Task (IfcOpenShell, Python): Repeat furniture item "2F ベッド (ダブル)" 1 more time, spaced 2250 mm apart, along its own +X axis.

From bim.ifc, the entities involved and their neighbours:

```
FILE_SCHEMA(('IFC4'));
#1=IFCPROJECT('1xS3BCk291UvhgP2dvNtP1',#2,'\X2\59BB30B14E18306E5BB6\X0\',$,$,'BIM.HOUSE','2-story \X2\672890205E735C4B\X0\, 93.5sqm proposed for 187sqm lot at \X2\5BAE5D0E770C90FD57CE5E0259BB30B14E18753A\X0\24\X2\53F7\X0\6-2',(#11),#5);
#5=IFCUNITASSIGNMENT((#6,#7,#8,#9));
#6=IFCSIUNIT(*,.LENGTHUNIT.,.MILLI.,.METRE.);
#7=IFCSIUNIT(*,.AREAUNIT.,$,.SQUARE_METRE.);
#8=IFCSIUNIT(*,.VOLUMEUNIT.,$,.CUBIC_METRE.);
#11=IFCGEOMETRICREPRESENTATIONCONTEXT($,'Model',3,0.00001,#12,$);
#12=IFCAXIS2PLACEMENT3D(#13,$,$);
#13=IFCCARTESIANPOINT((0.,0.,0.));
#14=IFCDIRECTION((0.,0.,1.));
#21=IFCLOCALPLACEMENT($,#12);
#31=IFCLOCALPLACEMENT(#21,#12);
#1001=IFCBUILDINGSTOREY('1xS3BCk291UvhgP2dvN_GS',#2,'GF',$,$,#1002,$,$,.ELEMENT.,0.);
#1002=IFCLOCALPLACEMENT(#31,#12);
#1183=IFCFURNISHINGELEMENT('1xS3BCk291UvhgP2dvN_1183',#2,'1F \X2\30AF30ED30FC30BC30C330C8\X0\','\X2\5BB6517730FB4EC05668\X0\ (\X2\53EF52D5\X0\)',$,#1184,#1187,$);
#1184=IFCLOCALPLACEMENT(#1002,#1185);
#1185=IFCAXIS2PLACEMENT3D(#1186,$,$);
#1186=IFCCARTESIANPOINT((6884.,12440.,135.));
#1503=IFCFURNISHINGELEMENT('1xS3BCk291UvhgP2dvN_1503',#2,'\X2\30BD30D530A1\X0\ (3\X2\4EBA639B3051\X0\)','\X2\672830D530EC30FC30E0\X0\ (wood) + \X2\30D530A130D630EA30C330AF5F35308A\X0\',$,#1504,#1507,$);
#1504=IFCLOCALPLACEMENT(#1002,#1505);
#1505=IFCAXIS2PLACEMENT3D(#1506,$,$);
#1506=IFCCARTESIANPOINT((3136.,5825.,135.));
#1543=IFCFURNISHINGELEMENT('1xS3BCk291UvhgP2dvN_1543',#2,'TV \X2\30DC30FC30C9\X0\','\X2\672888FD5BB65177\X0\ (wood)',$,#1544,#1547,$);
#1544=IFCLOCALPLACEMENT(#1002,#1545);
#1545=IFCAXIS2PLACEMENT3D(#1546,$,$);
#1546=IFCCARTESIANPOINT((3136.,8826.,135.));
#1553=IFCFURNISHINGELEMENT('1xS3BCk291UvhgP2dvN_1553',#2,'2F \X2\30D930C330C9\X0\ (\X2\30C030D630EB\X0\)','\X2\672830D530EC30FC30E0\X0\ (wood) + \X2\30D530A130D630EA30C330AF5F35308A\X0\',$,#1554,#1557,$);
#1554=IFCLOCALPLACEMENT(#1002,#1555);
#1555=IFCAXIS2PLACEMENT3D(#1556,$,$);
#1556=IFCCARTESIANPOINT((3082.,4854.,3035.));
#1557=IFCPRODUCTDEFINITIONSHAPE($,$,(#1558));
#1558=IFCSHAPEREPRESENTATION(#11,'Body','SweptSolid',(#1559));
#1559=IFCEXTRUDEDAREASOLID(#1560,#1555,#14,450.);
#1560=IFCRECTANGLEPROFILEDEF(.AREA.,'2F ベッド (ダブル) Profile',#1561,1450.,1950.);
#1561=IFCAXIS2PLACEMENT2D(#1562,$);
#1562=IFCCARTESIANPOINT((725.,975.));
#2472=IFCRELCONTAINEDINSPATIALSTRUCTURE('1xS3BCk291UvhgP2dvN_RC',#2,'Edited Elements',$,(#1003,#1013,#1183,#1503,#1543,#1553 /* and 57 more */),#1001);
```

```python
import ifcopenshell
import ifcopenshell.api.geometry
import ifcopenshell.api.root
import ifcopenshell.util.element
import ifcopenshell.util.placement

model = ifcopenshell.open("bim.ifc")


def reuse_history(source, copy):
    """copy_class also copies each property set's owner history, people and application; keep the originals."""
    for rel in copy.IsDefinedBy:
        if rel.is_a("IfcRelDefinesByProperties") and (history := rel.RelatingPropertyDefinition.OwnerHistory):
            rel.RelatingPropertyDefinition.OwnerHistory = source.OwnerHistory
            ifcopenshell.util.element.remove_deep2(model, history)


source = model.by_guid("1xS3BCk291UvhgP2dvN_1553")
base = ifcopenshell.util.placement.get_local_placement(source.ObjectPlacement)
step = base[:3, 0] * 2250.0

for i in range(1, 2):
    copy = ifcopenshell.api.root.copy_class(model, product=source)
    copy.Representation = ifcopenshell.util.element.copy_deep(
        model, source.Representation, exclude=["IfcGeometricRepresentationContext", "IfcRepresentationMap"]
    )
    reuse_history(source, copy)
    matrix = base.copy()
    matrix[:3, 3] += i * step
    print("added at", matrix[:3, 3].round(3) + 0.0)
    ifcopenshell.api.geometry.edit_object_placement(model, product=copy, matrix=matrix, is_si=False)

model.write("bim_v2.ifc")
```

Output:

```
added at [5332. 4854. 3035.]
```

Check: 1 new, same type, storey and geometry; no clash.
